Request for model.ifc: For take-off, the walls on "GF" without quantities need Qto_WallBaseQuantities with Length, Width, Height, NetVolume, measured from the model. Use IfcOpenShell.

First a look at what the model holds.

```python
import ifcopenshell
import ifcopenshell.util.element
import ifcopenshell.util.unit

model = ifcopenshell.open("model.ifc")
print(model.schema)
for unit_type in ("LENGTHUNIT", "AREAUNIT", "VOLUMEUNIT"):
    print(unit_type, ifcopenshell.util.unit.calculate_unit_scale(model, unit_type))
storey = next(s for s in model.by_type("IfcBuildingStorey") if s.Name == "GF")
walls = [e for e in ifcopenshell.util.element.get_decomposition(storey) if e.is_a("IfcWall")]
for e in sorted(walls, key=lambda e: e.id()):
    print(e.id(), e.is_a(), e.Name, list(ifcopenshell.util.element.get_psets(e, qtos_only=True)), sep=" | ")
```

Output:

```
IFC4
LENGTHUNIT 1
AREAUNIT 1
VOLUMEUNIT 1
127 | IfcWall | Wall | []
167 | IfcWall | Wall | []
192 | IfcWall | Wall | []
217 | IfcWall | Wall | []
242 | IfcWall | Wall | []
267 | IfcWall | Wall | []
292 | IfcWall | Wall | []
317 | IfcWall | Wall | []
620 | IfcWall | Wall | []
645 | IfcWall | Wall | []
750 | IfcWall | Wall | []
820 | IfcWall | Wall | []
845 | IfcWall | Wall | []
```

```python
import ifcopenshell
import ifcopenshell.api.pset
import ifcopenshell.geom
import ifcopenshell.util.element
import ifcopenshell.util.shape
import ifcopenshell.util.unit

model = ifcopenshell.open("model.ifc")
unit_scale = ifcopenshell.util.unit.calculate_unit_scale(model)
volume_scale = ifcopenshell.util.unit.calculate_unit_scale(model, "VOLUMEUNIT")
settings = ifcopenshell.geom.settings()

storey = next(s for s in model.by_type("IfcBuildingStorey") if s.Name == "GF")
walls = [e for e in ifcopenshell.util.element.get_decomposition(storey) if e.is_a("IfcWall")]

for e in sorted(walls, key=lambda e: e.id()):
    if ifcopenshell.util.element.get_psets(e, qtos_only=True, should_inherit=False):
        continue
    # Geometry comes back in metres, in the element's own axes.
    shape = ifcopenshell.geom.create_shape(settings, e)
    values = {
        "Length": ifcopenshell.util.shape.get_x(shape.geometry) / unit_scale,
        "Width": ifcopenshell.util.shape.get_y(shape.geometry) / unit_scale,
        "Height": ifcopenshell.util.shape.get_z(shape.geometry) / unit_scale,
        "NetVolume": ifcopenshell.util.shape.get_volume(shape.geometry) / volume_scale,
    }
    qto = ifcopenshell.api.pset.add_qto(model, product=e, name="Qto_WallBaseQuantities")
    ifcopenshell.api.pset.edit_qto(model, qto=qto, properties=values)
    print(e.id(), {k: round(v, 3) for k, v in values.items()})

model.write("model_edited.ifc")
```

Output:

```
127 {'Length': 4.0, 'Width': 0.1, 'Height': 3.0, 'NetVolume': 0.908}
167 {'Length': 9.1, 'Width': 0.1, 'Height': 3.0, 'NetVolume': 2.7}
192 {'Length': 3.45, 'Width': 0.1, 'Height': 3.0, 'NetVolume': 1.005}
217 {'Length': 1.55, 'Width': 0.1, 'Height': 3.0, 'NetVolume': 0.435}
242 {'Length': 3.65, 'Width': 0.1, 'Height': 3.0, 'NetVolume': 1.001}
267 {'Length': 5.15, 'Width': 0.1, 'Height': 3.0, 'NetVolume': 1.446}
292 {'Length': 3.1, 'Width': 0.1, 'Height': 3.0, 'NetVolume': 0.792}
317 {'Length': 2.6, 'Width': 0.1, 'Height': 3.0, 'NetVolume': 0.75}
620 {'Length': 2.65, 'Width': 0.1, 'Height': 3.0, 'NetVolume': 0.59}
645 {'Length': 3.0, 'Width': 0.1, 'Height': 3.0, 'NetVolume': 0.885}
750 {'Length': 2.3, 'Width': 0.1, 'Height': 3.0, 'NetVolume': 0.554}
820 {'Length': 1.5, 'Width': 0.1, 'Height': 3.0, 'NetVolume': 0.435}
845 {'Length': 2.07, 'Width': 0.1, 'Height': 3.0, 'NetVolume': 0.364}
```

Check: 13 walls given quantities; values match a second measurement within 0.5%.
